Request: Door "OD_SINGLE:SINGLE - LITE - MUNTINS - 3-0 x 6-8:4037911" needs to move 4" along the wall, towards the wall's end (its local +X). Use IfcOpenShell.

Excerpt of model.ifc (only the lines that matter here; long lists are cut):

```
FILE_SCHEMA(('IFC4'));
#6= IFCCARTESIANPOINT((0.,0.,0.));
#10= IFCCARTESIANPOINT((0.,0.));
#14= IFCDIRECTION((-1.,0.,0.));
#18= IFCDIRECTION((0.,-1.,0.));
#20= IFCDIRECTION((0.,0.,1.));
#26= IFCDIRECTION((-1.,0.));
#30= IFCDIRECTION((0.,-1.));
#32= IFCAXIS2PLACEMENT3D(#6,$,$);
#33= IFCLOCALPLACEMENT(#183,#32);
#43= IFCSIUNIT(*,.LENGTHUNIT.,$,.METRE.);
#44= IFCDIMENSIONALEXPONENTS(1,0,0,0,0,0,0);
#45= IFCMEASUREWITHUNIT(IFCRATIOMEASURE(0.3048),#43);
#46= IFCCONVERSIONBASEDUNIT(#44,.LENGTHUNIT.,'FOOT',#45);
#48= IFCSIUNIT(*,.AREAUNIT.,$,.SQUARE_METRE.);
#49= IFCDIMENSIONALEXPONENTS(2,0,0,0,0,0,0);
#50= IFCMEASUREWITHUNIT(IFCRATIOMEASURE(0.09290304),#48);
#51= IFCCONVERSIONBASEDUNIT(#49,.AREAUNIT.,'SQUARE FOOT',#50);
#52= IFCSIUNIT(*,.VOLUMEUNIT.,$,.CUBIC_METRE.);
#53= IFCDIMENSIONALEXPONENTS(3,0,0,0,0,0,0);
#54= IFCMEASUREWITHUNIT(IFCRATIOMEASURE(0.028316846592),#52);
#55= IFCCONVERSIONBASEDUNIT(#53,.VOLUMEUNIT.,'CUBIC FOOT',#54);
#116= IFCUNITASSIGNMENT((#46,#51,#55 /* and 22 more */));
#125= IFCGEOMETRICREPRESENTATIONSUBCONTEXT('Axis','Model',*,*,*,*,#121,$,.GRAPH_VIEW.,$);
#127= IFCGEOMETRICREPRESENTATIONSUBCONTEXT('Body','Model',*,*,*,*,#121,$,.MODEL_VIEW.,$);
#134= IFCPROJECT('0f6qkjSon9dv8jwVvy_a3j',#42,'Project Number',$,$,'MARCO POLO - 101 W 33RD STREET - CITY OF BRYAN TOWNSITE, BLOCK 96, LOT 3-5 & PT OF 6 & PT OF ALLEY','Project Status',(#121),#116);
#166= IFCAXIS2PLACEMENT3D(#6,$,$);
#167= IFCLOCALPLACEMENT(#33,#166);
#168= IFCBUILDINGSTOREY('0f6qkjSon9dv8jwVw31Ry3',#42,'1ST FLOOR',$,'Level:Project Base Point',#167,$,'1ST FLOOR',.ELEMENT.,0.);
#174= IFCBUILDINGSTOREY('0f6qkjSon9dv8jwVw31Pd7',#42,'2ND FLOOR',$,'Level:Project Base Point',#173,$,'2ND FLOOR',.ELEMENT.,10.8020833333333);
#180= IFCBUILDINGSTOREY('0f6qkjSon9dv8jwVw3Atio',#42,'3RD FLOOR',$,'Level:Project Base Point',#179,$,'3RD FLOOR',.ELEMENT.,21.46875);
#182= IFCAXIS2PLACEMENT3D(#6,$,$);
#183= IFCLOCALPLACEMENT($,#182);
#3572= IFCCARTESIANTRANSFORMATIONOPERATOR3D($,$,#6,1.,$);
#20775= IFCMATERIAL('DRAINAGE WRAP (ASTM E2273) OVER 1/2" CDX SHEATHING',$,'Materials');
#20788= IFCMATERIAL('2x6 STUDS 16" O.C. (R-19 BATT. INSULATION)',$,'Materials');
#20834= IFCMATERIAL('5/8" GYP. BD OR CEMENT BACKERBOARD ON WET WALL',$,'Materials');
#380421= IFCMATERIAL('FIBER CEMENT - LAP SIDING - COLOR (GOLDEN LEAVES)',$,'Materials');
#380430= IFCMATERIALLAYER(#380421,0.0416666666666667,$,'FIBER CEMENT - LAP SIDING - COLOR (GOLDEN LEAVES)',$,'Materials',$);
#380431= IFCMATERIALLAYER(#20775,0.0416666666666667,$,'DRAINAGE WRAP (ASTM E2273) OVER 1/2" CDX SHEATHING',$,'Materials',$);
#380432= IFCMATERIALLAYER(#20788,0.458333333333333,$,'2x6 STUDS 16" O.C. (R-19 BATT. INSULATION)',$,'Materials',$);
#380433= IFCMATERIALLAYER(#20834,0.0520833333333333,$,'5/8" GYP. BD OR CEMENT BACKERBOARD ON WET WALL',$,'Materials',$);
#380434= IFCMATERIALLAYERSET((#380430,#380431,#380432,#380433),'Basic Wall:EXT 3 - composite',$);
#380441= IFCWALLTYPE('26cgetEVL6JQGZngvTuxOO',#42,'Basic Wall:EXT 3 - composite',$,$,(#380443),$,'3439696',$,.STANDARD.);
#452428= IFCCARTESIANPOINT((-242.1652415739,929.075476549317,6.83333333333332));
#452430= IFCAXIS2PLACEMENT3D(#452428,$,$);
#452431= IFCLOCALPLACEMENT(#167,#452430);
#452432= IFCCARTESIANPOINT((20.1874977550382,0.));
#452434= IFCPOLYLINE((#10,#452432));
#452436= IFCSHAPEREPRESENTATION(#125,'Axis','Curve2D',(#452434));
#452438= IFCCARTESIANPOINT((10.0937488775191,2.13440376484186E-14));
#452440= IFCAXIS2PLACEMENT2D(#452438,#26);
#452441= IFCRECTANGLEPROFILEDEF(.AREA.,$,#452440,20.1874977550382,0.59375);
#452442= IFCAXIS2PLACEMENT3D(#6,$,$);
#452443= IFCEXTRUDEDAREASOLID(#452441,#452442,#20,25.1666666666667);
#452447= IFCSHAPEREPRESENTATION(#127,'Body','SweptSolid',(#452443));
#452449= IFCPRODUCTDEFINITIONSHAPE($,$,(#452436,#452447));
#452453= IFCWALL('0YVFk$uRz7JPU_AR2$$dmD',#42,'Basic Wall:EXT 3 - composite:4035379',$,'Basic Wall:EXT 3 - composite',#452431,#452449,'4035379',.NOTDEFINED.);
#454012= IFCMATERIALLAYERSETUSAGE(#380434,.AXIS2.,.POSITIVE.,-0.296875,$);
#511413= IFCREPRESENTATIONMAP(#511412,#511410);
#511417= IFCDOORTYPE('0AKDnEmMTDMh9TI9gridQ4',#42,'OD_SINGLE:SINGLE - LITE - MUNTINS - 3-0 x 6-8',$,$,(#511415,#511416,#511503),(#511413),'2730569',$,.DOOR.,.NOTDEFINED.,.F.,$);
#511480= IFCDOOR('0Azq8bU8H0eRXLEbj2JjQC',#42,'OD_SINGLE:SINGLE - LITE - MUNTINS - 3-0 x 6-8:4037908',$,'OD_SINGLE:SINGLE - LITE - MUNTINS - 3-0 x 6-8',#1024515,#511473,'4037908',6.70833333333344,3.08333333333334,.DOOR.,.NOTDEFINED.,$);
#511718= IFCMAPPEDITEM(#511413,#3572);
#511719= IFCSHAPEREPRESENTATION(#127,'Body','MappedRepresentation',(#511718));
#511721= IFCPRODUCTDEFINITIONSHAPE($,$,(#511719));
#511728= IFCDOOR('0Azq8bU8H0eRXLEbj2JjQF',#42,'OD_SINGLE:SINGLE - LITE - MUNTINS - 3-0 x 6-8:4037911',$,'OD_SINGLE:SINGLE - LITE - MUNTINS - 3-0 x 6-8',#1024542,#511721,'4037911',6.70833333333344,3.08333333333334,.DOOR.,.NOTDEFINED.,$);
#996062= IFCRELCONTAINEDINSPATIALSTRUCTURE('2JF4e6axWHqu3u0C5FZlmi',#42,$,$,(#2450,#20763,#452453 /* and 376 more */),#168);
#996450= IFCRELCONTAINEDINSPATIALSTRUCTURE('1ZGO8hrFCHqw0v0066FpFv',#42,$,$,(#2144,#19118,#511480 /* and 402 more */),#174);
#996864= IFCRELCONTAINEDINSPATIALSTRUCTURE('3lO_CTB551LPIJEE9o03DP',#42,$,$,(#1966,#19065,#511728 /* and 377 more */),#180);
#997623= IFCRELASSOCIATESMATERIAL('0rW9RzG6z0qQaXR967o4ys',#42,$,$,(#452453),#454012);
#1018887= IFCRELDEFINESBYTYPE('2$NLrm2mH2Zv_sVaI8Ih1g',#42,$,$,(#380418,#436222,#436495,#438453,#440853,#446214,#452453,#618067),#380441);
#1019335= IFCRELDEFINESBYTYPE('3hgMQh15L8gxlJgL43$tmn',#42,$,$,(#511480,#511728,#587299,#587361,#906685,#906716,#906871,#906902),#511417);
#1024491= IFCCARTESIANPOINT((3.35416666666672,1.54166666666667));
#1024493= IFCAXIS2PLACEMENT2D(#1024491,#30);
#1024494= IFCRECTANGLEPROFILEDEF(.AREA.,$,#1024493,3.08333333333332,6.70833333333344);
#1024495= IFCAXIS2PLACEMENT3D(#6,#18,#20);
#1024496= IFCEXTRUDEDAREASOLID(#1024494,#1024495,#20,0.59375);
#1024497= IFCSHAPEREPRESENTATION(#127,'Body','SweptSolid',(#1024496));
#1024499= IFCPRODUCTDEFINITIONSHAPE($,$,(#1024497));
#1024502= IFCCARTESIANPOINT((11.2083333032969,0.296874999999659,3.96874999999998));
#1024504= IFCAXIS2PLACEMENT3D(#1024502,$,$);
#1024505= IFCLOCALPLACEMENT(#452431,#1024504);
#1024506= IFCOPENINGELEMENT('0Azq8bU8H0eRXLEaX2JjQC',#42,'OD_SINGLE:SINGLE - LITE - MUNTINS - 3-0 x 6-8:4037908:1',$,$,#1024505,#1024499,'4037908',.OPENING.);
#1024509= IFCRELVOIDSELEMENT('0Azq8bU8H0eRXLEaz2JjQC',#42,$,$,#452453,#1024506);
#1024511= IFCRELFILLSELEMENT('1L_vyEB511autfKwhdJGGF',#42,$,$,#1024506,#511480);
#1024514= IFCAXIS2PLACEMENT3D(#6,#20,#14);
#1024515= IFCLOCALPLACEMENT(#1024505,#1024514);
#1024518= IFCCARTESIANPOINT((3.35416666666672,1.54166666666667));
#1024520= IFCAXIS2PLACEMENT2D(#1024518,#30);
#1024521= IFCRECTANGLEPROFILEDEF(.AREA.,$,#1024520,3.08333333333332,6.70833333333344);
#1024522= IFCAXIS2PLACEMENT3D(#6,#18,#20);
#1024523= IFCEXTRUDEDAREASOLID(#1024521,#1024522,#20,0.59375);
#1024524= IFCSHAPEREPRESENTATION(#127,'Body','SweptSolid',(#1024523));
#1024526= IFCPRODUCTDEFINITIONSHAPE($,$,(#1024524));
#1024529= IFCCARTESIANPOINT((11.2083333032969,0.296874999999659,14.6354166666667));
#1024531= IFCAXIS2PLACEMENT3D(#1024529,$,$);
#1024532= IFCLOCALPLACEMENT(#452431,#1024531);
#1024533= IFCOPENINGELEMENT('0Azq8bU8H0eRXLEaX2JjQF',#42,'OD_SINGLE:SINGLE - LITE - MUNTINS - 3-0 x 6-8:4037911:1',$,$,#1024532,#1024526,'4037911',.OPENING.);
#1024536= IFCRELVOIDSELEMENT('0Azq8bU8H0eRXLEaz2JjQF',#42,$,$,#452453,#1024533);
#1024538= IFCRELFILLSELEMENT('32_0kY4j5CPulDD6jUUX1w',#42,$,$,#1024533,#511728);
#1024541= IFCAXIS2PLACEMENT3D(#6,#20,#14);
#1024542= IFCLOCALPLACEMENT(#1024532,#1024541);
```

```python
import ifcopenshell
import ifcopenshell.api.geometry
import ifcopenshell.util.placement
import ifcopenshell.util.unit

model = ifcopenshell.open("model.ifc")
unit_scale = ifcopenshell.util.unit.calculate_unit_scale(model)

door = model.by_guid("0Azq8bU8H0eRXLEbj2JjQF")
opening = door.FillsVoids[0].RelatingOpeningElement
wall = opening.VoidsElements[0].RelatingBuildingElement

wall_matrix = ifcopenshell.util.placement.get_local_placement(wall.ObjectPlacement)
shift = wall_matrix[:3, 0] * 4 * 0.0254 / unit_scale
before = ifcopenshell.util.placement.get_local_placement(door.ObjectPlacement)[:3, 3].copy()

# The door is placed relative to its opening, so it follows when the opening moves.
matrix = ifcopenshell.util.placement.get_local_placement(opening.ObjectPlacement)
matrix[:3, 3] += shift
ifcopenshell.api.geometry.edit_object_placement(
    model, product=opening, matrix=matrix, is_si=False, should_transform_children=True
)

after = ifcopenshell.util.placement.get_local_placement(door.ObjectPlacement)[:3, 3]
print("door moved by", (after - before).round(3) + 0.0)

model.write("model_rev.ifc")
```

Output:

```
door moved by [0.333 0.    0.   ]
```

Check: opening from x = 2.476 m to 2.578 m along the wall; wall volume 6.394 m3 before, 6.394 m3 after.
